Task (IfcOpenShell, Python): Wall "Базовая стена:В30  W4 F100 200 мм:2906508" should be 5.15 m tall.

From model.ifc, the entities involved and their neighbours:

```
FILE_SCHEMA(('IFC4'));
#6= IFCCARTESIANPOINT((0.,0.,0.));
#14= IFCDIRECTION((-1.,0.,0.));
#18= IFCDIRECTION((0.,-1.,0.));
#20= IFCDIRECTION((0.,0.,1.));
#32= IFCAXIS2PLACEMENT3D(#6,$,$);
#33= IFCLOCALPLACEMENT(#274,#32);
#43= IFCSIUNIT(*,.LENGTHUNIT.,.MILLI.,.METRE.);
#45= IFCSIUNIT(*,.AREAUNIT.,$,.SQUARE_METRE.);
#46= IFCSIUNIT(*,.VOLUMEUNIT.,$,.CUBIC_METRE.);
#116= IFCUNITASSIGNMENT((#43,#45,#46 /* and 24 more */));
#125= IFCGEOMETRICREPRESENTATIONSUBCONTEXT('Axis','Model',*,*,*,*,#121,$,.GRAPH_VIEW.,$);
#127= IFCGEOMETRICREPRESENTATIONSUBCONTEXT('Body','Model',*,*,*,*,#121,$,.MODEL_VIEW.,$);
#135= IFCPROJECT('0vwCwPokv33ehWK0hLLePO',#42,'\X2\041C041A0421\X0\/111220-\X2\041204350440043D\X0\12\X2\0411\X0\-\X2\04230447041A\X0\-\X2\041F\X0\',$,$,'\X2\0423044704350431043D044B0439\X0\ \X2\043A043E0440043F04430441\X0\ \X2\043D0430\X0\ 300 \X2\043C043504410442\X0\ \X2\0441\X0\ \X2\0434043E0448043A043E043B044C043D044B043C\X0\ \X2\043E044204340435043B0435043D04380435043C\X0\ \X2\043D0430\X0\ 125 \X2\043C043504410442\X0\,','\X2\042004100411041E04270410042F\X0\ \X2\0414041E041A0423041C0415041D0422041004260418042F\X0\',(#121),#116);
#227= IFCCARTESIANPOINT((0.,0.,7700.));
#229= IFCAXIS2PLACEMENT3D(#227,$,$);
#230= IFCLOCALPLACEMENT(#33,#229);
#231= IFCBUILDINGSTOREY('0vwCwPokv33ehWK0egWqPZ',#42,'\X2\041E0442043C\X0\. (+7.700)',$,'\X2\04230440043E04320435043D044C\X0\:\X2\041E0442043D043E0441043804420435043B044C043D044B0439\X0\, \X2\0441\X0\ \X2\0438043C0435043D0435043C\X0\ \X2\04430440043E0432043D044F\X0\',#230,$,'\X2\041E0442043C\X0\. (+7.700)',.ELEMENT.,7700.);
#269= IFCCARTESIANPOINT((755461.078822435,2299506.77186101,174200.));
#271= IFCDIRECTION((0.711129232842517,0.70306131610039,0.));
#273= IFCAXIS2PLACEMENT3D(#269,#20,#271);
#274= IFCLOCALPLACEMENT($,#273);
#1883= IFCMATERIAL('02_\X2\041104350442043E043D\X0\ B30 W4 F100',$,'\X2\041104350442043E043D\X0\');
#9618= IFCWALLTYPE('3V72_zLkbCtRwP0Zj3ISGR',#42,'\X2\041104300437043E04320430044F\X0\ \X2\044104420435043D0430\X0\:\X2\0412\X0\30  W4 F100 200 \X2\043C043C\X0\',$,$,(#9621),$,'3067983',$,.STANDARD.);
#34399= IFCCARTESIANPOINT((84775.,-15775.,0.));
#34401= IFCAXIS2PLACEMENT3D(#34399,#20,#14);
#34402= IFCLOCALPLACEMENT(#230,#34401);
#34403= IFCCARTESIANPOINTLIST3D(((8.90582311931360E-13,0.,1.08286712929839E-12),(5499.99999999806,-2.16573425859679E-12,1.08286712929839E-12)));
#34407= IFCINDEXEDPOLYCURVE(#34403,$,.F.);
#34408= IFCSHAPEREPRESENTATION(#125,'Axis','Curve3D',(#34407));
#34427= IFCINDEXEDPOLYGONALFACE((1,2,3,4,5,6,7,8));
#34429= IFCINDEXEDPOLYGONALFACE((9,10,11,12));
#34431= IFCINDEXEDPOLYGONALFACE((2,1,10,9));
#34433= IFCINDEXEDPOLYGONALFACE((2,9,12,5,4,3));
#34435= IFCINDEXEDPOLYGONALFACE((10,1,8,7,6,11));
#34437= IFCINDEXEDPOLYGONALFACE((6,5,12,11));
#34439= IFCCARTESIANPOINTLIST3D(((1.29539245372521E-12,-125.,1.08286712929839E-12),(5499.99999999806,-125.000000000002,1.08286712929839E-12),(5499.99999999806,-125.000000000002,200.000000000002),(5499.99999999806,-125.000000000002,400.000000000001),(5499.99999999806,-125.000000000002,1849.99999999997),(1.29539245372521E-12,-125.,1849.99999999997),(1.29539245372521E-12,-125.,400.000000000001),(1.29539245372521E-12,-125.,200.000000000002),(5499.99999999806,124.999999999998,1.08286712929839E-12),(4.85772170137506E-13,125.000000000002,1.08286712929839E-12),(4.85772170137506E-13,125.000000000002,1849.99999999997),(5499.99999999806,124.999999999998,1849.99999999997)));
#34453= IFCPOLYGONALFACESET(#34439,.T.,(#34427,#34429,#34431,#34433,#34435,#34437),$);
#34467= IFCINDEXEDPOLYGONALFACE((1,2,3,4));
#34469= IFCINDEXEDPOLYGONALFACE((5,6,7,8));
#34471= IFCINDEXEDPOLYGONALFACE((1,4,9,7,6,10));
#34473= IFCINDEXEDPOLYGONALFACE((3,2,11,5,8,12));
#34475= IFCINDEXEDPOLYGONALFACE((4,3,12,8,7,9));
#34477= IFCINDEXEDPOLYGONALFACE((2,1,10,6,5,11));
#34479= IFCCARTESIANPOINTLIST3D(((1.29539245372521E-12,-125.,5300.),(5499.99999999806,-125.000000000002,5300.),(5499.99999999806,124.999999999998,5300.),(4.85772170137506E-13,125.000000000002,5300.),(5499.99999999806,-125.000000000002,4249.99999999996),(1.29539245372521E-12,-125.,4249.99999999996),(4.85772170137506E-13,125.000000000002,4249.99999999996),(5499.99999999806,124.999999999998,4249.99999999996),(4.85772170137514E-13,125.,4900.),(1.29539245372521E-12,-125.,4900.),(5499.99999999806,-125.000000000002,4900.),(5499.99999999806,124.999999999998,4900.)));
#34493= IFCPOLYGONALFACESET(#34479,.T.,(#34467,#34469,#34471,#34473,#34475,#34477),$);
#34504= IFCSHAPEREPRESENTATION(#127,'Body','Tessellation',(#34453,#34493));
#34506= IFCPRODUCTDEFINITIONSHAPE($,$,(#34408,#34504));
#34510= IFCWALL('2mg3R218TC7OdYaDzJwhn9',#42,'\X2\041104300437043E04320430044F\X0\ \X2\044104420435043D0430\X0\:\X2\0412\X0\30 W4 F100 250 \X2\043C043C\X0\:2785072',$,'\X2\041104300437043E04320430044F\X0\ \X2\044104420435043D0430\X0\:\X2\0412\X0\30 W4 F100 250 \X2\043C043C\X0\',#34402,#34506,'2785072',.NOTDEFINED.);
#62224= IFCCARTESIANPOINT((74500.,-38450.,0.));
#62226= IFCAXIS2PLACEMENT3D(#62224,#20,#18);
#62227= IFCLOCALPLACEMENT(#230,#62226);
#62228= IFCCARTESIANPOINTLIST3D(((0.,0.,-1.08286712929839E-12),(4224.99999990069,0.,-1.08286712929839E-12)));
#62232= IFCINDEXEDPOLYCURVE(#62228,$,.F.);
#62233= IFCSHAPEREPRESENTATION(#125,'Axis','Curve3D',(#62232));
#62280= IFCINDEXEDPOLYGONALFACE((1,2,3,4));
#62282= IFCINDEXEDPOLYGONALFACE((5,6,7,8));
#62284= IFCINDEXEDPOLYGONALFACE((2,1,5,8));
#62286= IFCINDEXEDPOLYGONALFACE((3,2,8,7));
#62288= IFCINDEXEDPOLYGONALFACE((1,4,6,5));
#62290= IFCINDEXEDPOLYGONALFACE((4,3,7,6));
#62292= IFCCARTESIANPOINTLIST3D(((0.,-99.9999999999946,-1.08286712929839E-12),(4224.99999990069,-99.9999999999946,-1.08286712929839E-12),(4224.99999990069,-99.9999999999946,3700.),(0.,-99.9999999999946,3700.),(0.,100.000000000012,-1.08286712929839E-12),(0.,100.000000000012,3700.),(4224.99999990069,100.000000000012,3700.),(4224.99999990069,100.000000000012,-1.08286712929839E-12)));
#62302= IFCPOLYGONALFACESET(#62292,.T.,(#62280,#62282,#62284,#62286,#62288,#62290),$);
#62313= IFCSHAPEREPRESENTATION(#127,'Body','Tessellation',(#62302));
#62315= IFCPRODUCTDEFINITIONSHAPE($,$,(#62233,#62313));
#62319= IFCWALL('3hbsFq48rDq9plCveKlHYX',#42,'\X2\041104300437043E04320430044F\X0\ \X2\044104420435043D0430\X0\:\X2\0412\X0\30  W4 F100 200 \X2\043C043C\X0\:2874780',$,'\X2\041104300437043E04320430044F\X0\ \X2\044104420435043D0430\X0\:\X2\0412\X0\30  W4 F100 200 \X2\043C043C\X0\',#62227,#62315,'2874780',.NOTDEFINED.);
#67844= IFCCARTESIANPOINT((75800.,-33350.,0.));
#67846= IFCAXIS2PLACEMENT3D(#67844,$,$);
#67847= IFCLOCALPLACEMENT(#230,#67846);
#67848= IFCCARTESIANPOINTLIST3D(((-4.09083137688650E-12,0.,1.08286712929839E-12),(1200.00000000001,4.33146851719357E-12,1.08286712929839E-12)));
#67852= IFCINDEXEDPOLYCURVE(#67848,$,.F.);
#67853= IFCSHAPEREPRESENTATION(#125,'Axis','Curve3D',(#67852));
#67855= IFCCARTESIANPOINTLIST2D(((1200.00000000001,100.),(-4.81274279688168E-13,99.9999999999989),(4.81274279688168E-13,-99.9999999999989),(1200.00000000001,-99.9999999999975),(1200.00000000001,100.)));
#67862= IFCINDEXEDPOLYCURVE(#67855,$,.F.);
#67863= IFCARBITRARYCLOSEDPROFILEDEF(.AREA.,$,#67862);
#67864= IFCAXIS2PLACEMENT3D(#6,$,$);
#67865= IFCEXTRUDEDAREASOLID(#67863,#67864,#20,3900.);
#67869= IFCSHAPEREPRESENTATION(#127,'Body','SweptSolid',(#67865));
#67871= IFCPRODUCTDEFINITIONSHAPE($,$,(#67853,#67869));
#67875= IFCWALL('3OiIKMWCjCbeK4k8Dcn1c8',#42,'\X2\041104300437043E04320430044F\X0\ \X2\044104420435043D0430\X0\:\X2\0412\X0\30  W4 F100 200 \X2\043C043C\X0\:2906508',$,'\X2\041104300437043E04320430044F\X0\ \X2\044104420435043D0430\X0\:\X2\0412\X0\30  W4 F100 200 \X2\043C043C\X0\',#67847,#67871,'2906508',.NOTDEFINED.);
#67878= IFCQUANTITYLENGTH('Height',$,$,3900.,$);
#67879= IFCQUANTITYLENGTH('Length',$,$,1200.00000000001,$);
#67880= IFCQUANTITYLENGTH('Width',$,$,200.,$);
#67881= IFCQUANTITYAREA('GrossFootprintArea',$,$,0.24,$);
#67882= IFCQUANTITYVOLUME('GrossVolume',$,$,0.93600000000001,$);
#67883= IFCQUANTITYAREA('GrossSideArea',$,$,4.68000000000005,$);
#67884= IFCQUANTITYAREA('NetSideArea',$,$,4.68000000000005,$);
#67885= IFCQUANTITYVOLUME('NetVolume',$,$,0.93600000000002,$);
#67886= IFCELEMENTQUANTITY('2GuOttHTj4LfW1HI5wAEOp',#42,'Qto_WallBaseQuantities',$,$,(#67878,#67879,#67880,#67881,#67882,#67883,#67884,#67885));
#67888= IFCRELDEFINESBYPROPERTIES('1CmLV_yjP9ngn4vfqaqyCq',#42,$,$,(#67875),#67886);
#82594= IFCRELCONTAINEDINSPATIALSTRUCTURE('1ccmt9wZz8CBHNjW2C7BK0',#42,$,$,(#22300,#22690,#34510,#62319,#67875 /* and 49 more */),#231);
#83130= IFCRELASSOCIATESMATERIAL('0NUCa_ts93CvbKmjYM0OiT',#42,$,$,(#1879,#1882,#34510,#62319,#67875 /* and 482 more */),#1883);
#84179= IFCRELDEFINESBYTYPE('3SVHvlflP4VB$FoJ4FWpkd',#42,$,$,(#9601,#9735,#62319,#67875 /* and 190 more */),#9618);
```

```python
import ifcopenshell
import ifcopenshell.api.pset
import ifcopenshell.geom
import ifcopenshell.util.element
import ifcopenshell.util.representation
import ifcopenshell.util.shape
import ifcopenshell.util.unit

model = ifcopenshell.open("model.ifc")
unit_scale = ifcopenshell.util.unit.calculate_unit_scale(model)
area_scale = ifcopenshell.util.unit.calculate_unit_scale(model, "AREAUNIT")
volume_scale = ifcopenshell.util.unit.calculate_unit_scale(model, "VOLUMEUNIT")
settings = ifcopenshell.geom.settings()


def volume(element):
    """Net volume in cubic metres, openings subtracted."""
    shape = ifcopenshell.geom.create_shape(settings, element)
    return ifcopenshell.util.shape.get_volume(shape.geometry)


wall = model.by_guid("3OiIKMWCjCbeK4k8Dcn1c8")
before = volume(wall)

body = ifcopenshell.util.representation.get_representation(wall, "Model", "Body")
solid = body.Items[0]
old_height = solid.Depth
solid.Depth = 5.15 / unit_scale
after = volume(wall)
thickness = 0.2  # wall thickness in metres

# Update the stored height, areas and volumes.
qto = model.by_id(ifcopenshell.util.element.get_pset(wall, "Qto_WallBaseQuantities", should_inherit=False)["id"])
ifcopenshell.api.pset.edit_qto(model, qto=qto, properties={
    "Height": solid.Depth,
    "GrossVolume": ifcopenshell.util.element.get_pset(wall, "Qto_WallBaseQuantities", "GrossVolume") * solid.Depth / old_height,
    "GrossSideArea": ifcopenshell.util.element.get_pset(wall, "Qto_WallBaseQuantities", "GrossSideArea") * solid.Depth / old_height,
    "NetSideArea": after / thickness / area_scale,
    "NetVolume": after / volume_scale,
})

print(f"height {old_height:g} -> {solid.Depth:g}, volume {before:.3f} -> {after:.3f} m3")

model.write("model_updated.ifc")
```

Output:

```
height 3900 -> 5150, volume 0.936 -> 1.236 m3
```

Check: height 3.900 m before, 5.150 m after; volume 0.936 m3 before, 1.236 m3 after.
